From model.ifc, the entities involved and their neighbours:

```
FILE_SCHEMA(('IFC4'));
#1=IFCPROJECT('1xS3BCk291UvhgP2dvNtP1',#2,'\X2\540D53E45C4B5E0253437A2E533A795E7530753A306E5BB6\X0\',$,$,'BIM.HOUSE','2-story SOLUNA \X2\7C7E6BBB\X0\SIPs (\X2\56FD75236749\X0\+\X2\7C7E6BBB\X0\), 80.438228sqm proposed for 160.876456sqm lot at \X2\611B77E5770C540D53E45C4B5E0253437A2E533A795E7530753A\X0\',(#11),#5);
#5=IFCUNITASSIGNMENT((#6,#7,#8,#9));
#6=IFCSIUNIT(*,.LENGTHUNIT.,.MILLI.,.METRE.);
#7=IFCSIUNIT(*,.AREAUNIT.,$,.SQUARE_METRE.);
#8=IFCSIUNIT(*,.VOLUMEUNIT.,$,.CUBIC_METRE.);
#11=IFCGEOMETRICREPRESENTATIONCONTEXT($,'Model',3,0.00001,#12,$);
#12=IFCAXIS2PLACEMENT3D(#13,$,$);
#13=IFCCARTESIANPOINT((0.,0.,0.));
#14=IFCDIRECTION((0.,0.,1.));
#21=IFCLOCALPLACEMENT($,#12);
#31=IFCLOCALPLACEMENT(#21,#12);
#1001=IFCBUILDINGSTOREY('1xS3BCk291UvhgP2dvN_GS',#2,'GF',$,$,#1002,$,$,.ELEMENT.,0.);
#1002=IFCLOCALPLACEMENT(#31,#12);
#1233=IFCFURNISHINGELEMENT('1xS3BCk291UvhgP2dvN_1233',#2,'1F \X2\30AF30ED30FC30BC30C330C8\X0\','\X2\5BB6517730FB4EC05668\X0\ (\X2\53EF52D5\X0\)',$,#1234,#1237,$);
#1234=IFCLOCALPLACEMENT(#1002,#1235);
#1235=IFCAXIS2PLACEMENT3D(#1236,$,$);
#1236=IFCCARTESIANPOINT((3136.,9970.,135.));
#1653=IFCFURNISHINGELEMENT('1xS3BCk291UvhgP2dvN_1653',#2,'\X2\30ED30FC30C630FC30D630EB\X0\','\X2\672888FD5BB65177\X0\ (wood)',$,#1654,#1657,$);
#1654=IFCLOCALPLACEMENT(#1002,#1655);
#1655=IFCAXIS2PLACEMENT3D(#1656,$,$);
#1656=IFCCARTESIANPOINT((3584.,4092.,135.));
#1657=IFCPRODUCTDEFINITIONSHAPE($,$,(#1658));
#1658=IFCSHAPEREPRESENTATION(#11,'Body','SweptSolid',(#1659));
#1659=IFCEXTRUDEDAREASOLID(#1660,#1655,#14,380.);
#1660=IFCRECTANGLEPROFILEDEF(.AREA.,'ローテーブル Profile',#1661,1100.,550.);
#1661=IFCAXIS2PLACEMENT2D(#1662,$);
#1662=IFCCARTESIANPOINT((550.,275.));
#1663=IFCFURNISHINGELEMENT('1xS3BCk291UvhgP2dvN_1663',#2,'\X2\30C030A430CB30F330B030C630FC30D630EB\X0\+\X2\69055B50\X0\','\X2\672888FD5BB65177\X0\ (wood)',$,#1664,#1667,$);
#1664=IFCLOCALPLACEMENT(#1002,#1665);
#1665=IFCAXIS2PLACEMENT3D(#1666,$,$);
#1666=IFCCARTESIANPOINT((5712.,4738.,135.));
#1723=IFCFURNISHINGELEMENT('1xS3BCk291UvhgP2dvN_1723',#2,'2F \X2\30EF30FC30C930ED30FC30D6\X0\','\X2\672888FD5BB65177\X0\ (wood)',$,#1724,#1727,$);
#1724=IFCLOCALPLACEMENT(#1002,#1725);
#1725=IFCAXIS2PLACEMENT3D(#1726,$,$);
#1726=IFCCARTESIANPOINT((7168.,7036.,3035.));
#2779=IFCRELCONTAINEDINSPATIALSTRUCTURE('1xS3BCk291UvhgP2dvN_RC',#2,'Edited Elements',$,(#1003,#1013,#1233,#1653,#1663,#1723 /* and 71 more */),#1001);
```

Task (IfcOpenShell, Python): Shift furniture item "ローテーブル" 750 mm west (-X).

```python
import ifcopenshell
import ifcopenshell.api.geometry
import ifcopenshell.util.placement
import ifcopenshell.util.unit

model = ifcopenshell.open("model.ifc")
unit_scale = ifcopenshell.util.unit.calculate_unit_scale(model)

item = model.by_guid("1xS3BCk291UvhgP2dvN_1653")
matrix = ifcopenshell.util.placement.get_local_placement(item.ObjectPlacement)
matrix[0, 3] -= 0.75 / unit_scale
ifcopenshell.api.geometry.edit_object_placement(model, product=item, matrix=matrix, is_si=False)

print(ifcopenshell.util.placement.get_local_placement(item.ObjectPlacement).round(3) + 0.0)

model.write("model-out.ifc")
```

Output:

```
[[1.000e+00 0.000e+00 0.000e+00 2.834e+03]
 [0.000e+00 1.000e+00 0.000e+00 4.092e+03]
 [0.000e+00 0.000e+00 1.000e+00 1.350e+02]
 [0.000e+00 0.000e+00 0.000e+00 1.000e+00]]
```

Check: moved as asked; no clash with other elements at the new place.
